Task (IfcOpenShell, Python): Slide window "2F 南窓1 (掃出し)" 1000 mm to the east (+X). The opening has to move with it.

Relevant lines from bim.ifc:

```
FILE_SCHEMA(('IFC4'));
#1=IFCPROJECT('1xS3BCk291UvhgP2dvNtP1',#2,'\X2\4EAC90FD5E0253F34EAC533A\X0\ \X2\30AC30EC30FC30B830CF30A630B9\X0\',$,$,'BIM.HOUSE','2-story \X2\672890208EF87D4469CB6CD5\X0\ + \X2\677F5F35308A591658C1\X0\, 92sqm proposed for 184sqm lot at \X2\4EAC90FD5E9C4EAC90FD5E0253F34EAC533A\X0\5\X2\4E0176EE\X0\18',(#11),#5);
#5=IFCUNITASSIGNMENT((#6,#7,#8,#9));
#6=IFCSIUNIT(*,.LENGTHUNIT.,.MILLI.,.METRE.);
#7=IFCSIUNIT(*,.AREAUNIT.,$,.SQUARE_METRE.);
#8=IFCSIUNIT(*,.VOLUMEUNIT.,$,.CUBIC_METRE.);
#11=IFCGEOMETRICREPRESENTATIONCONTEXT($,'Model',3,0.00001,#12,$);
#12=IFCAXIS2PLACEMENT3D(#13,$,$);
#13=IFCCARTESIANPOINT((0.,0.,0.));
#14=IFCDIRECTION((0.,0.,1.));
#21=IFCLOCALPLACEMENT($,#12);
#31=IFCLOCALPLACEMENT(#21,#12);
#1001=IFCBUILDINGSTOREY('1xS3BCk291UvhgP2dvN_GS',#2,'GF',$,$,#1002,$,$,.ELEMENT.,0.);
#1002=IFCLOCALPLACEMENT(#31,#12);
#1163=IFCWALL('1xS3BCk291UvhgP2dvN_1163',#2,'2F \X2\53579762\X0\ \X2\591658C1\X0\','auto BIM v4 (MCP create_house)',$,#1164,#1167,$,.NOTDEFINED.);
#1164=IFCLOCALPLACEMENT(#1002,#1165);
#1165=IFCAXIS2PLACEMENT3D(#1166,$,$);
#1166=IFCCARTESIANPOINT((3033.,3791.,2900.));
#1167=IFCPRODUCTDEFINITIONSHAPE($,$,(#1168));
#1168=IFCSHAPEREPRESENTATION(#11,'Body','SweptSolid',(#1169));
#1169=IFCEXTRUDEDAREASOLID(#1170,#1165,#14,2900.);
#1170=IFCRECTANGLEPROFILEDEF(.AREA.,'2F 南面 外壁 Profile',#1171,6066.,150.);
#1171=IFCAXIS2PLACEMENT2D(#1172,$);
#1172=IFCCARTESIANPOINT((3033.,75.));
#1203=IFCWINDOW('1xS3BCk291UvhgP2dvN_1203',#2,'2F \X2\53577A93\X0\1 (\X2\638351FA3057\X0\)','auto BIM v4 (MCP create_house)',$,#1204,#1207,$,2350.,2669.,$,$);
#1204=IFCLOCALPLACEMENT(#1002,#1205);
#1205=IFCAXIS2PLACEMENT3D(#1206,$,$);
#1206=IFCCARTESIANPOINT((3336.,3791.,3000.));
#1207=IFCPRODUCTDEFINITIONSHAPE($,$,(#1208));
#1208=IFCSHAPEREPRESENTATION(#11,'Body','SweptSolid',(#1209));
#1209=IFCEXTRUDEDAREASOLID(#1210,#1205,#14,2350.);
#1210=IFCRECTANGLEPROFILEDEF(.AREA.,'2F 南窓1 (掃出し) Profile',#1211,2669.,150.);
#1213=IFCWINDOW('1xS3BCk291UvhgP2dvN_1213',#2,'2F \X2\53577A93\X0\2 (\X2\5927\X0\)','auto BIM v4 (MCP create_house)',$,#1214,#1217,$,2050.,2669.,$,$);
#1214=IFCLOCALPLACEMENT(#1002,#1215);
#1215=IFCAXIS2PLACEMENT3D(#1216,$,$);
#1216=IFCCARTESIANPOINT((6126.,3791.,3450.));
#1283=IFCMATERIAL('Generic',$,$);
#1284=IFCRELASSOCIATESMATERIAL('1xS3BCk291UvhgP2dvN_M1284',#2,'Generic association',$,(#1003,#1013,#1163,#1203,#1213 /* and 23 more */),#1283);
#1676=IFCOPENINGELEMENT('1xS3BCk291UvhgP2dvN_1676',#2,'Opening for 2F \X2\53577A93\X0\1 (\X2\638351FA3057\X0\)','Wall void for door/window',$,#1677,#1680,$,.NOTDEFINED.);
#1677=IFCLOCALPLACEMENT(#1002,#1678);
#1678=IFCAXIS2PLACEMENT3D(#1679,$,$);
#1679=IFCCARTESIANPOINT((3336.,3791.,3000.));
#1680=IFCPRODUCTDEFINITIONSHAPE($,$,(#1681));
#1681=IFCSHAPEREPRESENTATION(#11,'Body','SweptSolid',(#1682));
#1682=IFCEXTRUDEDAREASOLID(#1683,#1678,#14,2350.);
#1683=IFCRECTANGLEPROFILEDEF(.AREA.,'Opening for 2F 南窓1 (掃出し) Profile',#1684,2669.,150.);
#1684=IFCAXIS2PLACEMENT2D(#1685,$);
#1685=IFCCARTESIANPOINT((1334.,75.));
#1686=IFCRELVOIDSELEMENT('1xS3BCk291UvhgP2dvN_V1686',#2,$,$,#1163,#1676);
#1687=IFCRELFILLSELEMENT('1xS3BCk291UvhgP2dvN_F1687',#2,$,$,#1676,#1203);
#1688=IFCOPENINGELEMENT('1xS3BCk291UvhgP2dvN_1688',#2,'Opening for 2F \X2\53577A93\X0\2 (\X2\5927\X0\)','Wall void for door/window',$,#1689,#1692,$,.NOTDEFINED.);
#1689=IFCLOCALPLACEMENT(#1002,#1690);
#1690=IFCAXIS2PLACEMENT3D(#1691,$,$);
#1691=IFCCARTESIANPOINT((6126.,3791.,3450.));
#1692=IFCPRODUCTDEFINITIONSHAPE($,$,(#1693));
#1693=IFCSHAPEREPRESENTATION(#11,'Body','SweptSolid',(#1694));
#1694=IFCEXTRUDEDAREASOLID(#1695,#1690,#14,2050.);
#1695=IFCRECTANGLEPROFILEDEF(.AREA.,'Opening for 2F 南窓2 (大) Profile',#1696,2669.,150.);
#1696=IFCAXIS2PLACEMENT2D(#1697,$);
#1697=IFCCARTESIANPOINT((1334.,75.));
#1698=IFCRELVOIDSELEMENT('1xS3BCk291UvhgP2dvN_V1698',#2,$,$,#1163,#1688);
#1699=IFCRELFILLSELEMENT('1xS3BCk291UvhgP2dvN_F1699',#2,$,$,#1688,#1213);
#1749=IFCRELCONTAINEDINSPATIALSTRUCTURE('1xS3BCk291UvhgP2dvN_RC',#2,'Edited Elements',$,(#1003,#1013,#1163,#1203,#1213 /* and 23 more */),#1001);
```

```python
import ifcopenshell
import ifcopenshell.api.geometry
import ifcopenshell.util.placement

model = ifcopenshell.open("bim.ifc")

window = model.by_guid("1xS3BCk291UvhgP2dvN_1203")
opening = window.FillsVoids[0].RelatingOpeningElement
wall = opening.VoidsElements[0].RelatingBuildingElement

wall_matrix = ifcopenshell.util.placement.get_local_placement(wall.ObjectPlacement)
shift = wall_matrix[:3, 0] * 1000.0
before = ifcopenshell.util.placement.get_local_placement(window.ObjectPlacement)[:3, 3].copy()

# The window is not placed relative to its opening, so move both.
for product in (opening, window):
    matrix = ifcopenshell.util.placement.get_local_placement(product.ObjectPlacement)
    matrix[:3, 3] += shift
    ifcopenshell.api.geometry.edit_object_placement(model, product=product, matrix=matrix, is_si=False)

after = ifcopenshell.util.placement.get_local_placement(window.ObjectPlacement)[:3, 3]
print("window moved by", (after - before).round(3) + 0.0)

model.write("bim_v2.ifc")
```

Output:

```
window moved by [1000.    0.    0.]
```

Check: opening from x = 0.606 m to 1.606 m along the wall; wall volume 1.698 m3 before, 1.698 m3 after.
